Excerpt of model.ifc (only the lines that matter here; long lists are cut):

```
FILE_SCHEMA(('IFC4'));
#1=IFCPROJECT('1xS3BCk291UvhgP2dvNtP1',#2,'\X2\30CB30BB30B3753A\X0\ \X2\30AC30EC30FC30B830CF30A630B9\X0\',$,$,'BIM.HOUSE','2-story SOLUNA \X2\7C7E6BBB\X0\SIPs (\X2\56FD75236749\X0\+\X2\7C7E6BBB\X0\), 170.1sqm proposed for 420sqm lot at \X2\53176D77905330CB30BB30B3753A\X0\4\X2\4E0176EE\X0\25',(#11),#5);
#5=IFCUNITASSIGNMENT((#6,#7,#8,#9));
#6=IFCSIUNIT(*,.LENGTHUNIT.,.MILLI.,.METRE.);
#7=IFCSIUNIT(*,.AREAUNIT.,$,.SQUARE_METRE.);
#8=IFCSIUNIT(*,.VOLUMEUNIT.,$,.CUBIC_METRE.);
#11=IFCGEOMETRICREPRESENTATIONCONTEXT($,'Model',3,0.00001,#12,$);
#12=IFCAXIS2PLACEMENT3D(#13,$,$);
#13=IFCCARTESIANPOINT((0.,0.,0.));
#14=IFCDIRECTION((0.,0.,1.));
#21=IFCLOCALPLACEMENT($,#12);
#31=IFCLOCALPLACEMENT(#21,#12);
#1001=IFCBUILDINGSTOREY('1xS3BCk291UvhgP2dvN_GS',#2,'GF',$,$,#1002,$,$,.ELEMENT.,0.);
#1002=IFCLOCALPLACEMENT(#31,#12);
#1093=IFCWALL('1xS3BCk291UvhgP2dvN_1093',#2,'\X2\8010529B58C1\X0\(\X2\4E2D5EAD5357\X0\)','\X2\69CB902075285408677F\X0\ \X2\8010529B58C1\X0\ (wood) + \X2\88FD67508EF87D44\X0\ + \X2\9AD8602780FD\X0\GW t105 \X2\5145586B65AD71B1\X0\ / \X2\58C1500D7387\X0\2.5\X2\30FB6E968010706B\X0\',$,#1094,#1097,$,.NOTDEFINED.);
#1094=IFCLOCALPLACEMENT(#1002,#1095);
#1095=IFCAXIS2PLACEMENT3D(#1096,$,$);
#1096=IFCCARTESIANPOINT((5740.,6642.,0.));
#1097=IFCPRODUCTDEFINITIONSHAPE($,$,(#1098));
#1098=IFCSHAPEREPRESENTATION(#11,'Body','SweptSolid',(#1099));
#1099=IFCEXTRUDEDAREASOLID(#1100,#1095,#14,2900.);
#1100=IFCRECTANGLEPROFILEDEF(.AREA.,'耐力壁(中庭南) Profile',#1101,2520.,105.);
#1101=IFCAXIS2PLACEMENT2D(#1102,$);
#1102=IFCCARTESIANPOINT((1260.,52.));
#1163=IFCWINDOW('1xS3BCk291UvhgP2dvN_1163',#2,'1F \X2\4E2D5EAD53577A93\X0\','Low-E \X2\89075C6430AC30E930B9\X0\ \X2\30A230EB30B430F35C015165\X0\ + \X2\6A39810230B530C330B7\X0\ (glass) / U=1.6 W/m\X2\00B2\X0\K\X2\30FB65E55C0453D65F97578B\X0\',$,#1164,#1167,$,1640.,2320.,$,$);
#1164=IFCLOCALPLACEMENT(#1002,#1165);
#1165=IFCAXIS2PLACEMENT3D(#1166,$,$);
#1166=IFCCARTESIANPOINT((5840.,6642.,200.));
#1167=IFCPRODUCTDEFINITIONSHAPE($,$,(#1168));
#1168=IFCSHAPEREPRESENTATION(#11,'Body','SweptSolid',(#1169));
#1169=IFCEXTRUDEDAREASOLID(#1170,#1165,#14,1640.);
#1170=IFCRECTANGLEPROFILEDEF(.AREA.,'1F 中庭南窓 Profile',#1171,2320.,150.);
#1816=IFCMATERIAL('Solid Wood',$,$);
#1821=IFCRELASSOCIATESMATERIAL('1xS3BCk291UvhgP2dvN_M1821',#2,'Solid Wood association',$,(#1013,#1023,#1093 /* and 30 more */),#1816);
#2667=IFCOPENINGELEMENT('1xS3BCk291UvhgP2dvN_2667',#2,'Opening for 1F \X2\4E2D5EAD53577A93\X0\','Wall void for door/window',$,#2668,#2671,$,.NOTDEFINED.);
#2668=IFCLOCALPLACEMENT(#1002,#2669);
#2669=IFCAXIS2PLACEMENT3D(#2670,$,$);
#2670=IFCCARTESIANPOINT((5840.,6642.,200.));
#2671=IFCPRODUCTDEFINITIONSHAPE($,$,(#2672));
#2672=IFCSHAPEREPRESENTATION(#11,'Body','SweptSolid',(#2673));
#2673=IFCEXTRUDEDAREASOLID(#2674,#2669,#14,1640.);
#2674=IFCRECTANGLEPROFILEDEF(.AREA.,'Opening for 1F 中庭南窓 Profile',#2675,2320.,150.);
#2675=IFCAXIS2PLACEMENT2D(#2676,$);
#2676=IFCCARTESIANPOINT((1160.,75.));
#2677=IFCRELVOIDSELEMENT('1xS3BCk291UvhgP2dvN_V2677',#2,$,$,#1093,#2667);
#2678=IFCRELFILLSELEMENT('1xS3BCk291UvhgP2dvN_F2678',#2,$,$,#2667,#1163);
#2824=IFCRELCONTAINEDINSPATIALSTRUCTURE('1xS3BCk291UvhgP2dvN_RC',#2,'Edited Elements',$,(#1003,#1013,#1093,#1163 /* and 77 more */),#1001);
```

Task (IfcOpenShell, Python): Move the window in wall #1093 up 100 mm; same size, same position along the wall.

```python
import numpy as np
import ifcopenshell
import ifcopenshell.api.geometry
import ifcopenshell.util.placement
import ifcopenshell.util.unit

model = ifcopenshell.open("model.ifc")
unit_scale = ifcopenshell.util.unit.calculate_unit_scale(model)

window = model.by_id(1163)
opening = window.FillsVoids[0].RelatingOpeningElement
dz = 100.0

shift = np.array([0.0, 0.0, dz])
# The window is not placed relative to its opening, so move both.
for product in (opening, window):
    matrix = ifcopenshell.util.placement.get_local_placement(product.ObjectPlacement)
    matrix[:3, 3] += shift
    ifcopenshell.api.geometry.edit_object_placement(model, product=product, matrix=matrix, is_si=False)

print(f"moved by {dz * unit_scale:+.3f} m")

model.write("model-out.ifc")
```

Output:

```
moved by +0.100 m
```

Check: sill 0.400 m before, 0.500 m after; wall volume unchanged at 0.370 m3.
